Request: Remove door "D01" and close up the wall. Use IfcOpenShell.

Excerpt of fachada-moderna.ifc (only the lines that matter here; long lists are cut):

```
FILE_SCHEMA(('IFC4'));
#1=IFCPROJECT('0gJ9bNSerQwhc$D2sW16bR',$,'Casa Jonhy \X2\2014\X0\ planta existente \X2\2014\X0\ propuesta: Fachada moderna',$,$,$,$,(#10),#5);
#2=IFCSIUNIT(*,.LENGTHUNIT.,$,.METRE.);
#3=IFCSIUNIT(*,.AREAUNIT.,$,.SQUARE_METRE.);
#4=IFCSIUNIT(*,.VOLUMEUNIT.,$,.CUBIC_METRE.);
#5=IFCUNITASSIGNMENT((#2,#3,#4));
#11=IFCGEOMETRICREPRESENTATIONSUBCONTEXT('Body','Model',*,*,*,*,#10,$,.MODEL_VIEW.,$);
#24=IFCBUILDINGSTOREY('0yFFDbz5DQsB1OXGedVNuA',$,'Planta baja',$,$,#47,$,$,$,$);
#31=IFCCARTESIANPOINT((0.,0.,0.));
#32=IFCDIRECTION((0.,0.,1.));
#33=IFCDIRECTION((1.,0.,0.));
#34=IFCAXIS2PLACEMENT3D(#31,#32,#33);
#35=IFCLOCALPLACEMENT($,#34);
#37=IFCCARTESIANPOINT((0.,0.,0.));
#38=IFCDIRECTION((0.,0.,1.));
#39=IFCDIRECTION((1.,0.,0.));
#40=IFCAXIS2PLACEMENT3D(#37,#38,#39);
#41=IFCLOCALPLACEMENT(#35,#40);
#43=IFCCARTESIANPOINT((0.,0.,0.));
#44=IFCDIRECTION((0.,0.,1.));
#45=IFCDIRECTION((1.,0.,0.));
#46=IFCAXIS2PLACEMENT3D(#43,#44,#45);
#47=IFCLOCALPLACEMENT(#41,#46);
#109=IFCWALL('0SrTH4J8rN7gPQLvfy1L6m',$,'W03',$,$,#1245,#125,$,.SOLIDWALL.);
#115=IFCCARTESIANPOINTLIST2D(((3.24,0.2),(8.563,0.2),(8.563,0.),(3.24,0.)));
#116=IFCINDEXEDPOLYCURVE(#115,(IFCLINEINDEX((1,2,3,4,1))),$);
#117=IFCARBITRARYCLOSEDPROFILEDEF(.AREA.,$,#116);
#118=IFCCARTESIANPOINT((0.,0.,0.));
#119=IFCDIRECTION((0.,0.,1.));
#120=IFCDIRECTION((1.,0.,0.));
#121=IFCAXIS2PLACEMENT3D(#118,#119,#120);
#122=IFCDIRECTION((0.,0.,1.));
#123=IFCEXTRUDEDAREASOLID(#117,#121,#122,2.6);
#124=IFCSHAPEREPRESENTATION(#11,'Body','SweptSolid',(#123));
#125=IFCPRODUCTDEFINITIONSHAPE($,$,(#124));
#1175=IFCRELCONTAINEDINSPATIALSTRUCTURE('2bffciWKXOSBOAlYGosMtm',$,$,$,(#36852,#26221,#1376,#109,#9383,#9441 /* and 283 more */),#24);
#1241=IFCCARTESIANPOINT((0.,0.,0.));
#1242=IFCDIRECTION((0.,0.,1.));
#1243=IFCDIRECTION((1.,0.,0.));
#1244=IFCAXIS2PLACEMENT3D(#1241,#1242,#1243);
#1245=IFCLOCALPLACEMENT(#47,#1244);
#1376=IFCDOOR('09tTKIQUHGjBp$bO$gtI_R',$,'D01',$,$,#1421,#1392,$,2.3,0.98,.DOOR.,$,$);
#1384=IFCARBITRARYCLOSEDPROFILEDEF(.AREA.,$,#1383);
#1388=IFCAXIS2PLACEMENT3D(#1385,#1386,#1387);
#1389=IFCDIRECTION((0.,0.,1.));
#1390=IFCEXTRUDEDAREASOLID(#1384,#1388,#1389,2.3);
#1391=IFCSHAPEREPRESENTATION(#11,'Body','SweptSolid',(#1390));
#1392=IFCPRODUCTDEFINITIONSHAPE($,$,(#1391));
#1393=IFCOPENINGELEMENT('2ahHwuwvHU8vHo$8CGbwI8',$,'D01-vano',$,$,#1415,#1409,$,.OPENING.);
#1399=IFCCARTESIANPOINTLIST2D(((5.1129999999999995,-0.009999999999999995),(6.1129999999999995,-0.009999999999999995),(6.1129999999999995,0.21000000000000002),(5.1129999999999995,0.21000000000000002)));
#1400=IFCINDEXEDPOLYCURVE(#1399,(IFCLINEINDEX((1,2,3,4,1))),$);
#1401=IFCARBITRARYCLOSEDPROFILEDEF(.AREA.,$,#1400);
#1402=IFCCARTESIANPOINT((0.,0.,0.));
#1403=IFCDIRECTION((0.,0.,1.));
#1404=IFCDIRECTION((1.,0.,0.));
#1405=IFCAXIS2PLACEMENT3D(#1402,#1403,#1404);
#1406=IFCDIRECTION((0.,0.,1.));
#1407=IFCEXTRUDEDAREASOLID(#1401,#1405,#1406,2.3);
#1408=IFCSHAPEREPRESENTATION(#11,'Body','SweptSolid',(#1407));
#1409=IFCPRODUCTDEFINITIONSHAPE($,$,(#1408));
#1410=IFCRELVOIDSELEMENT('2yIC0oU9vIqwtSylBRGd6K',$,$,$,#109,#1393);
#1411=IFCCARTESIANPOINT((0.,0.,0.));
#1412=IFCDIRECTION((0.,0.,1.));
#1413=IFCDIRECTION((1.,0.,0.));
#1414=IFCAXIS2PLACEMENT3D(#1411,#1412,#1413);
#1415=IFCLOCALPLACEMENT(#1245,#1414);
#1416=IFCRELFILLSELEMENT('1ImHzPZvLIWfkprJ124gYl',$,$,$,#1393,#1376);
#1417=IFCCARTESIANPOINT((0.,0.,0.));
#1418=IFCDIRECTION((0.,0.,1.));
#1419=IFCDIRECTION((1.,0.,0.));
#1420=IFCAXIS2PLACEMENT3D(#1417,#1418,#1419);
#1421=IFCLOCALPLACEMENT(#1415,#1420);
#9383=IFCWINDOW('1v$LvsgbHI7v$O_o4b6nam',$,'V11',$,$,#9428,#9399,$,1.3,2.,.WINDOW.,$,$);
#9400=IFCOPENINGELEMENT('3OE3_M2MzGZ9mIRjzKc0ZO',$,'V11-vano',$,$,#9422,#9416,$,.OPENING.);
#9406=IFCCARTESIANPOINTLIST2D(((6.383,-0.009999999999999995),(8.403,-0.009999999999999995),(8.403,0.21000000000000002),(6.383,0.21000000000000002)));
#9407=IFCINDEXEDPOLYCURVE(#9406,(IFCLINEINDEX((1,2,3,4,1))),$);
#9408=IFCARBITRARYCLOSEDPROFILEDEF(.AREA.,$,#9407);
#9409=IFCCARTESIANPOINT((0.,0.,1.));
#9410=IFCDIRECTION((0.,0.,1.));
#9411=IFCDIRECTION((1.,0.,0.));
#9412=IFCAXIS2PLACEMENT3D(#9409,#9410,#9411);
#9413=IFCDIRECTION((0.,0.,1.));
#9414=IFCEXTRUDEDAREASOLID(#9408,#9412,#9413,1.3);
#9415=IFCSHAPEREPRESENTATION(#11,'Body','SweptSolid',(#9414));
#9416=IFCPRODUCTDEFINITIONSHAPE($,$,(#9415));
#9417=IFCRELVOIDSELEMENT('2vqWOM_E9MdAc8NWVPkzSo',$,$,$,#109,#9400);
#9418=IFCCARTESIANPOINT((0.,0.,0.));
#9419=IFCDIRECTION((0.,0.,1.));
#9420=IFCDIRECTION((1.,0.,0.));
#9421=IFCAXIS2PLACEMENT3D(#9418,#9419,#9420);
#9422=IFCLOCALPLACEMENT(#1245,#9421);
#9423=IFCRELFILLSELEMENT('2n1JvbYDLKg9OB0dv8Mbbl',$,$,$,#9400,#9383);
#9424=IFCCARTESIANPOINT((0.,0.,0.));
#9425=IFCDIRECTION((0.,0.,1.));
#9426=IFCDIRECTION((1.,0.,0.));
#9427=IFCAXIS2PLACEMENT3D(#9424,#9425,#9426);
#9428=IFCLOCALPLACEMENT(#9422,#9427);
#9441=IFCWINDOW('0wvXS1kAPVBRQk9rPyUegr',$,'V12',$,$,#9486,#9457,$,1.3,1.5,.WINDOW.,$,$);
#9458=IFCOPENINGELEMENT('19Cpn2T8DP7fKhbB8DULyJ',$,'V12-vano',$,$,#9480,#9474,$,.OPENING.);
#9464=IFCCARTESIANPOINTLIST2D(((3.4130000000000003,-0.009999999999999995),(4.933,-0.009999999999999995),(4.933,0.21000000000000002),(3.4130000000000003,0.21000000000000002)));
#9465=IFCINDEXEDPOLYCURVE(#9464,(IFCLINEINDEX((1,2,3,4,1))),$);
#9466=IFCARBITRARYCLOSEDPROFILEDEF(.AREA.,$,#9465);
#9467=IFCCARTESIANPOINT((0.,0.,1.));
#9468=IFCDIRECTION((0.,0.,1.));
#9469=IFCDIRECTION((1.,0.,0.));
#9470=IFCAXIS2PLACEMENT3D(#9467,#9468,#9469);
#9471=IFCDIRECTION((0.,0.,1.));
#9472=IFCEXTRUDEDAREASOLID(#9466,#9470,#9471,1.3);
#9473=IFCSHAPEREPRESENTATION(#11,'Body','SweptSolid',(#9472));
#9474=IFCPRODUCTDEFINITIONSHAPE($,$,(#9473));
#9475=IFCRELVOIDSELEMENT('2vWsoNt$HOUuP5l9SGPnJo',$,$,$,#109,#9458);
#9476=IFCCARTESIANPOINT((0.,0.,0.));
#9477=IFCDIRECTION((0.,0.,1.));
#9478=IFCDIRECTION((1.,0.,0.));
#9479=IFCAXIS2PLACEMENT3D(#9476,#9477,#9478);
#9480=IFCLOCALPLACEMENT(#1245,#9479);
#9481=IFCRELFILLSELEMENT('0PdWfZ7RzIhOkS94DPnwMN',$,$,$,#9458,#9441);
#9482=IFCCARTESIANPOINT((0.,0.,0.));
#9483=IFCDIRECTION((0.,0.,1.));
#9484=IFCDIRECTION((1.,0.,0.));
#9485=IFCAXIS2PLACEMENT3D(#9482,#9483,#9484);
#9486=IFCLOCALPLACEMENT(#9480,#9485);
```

```python
import ifcopenshell
import ifcopenshell.api.feature
import ifcopenshell.api.root
import ifcopenshell.geom
import ifcopenshell.util.shape

model = ifcopenshell.open("fachada-moderna.ifc")
settings = ifcopenshell.geom.settings()


def volume(element):
    """Net volume in cubic metres, openings subtracted."""
    shape = ifcopenshell.geom.create_shape(settings, element)
    return ifcopenshell.util.shape.get_volume(shape.geometry)


door = model.by_guid("09tTKIQUHGjBp$bO$gtI_R")
opening = door.FillsVoids[0].RelatingOpeningElement
wall = opening.VoidsElements[0].RelatingBuildingElement
before = volume(wall)

ifcopenshell.api.root.remove_product(model, product=door)
ifcopenshell.api.feature.remove_feature(model, feature=opening)

after = volume(wall)

print(f"wall volume {before:.3f} -> {after:.3f} m3")

model.write("fachada-moderna-out.ifc")
```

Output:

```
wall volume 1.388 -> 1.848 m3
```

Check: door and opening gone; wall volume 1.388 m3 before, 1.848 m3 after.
